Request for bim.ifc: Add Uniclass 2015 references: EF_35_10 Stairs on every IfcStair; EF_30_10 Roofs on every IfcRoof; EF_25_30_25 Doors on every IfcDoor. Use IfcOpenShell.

First a look at what the model holds.

```python
import ifcopenshell

model = ifcopenshell.open("bim.ifc")
print(model.schema)
print("classifications:", [c.Name for c in model.by_type("IfcClassification")])
for ifc_class in ("IfcDoor", "IfcRoof", "IfcStair", "IfcWall", "IfcWindow"):
    print(ifc_class, len(model.by_type(ifc_class)))
```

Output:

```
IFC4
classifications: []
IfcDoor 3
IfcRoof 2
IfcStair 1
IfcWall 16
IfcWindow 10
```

```python
import ifcopenshell
import ifcopenshell.api.classification

model = ifcopenshell.open("bim.ifc")

system = ifcopenshell.api.classification.add_classification(model, classification="Uniclass 2015")

codes = {
    "IfcStair": ("EF_35_10", "Stairs"),
    "IfcRoof": ("EF_30_10", "Roofs"),
    "IfcDoor": ("EF_25_30_25", "Doors"),
}
for ifc_class, (code, name) in codes.items():
    products = model.by_type(ifc_class)
    ifcopenshell.api.classification.add_reference(
        model, products=products, classification=system, identification=code, name=name
    )
    print(code, len(products))

model.write("bim_updated.ifc")
```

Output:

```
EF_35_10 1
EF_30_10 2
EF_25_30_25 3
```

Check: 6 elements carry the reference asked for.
